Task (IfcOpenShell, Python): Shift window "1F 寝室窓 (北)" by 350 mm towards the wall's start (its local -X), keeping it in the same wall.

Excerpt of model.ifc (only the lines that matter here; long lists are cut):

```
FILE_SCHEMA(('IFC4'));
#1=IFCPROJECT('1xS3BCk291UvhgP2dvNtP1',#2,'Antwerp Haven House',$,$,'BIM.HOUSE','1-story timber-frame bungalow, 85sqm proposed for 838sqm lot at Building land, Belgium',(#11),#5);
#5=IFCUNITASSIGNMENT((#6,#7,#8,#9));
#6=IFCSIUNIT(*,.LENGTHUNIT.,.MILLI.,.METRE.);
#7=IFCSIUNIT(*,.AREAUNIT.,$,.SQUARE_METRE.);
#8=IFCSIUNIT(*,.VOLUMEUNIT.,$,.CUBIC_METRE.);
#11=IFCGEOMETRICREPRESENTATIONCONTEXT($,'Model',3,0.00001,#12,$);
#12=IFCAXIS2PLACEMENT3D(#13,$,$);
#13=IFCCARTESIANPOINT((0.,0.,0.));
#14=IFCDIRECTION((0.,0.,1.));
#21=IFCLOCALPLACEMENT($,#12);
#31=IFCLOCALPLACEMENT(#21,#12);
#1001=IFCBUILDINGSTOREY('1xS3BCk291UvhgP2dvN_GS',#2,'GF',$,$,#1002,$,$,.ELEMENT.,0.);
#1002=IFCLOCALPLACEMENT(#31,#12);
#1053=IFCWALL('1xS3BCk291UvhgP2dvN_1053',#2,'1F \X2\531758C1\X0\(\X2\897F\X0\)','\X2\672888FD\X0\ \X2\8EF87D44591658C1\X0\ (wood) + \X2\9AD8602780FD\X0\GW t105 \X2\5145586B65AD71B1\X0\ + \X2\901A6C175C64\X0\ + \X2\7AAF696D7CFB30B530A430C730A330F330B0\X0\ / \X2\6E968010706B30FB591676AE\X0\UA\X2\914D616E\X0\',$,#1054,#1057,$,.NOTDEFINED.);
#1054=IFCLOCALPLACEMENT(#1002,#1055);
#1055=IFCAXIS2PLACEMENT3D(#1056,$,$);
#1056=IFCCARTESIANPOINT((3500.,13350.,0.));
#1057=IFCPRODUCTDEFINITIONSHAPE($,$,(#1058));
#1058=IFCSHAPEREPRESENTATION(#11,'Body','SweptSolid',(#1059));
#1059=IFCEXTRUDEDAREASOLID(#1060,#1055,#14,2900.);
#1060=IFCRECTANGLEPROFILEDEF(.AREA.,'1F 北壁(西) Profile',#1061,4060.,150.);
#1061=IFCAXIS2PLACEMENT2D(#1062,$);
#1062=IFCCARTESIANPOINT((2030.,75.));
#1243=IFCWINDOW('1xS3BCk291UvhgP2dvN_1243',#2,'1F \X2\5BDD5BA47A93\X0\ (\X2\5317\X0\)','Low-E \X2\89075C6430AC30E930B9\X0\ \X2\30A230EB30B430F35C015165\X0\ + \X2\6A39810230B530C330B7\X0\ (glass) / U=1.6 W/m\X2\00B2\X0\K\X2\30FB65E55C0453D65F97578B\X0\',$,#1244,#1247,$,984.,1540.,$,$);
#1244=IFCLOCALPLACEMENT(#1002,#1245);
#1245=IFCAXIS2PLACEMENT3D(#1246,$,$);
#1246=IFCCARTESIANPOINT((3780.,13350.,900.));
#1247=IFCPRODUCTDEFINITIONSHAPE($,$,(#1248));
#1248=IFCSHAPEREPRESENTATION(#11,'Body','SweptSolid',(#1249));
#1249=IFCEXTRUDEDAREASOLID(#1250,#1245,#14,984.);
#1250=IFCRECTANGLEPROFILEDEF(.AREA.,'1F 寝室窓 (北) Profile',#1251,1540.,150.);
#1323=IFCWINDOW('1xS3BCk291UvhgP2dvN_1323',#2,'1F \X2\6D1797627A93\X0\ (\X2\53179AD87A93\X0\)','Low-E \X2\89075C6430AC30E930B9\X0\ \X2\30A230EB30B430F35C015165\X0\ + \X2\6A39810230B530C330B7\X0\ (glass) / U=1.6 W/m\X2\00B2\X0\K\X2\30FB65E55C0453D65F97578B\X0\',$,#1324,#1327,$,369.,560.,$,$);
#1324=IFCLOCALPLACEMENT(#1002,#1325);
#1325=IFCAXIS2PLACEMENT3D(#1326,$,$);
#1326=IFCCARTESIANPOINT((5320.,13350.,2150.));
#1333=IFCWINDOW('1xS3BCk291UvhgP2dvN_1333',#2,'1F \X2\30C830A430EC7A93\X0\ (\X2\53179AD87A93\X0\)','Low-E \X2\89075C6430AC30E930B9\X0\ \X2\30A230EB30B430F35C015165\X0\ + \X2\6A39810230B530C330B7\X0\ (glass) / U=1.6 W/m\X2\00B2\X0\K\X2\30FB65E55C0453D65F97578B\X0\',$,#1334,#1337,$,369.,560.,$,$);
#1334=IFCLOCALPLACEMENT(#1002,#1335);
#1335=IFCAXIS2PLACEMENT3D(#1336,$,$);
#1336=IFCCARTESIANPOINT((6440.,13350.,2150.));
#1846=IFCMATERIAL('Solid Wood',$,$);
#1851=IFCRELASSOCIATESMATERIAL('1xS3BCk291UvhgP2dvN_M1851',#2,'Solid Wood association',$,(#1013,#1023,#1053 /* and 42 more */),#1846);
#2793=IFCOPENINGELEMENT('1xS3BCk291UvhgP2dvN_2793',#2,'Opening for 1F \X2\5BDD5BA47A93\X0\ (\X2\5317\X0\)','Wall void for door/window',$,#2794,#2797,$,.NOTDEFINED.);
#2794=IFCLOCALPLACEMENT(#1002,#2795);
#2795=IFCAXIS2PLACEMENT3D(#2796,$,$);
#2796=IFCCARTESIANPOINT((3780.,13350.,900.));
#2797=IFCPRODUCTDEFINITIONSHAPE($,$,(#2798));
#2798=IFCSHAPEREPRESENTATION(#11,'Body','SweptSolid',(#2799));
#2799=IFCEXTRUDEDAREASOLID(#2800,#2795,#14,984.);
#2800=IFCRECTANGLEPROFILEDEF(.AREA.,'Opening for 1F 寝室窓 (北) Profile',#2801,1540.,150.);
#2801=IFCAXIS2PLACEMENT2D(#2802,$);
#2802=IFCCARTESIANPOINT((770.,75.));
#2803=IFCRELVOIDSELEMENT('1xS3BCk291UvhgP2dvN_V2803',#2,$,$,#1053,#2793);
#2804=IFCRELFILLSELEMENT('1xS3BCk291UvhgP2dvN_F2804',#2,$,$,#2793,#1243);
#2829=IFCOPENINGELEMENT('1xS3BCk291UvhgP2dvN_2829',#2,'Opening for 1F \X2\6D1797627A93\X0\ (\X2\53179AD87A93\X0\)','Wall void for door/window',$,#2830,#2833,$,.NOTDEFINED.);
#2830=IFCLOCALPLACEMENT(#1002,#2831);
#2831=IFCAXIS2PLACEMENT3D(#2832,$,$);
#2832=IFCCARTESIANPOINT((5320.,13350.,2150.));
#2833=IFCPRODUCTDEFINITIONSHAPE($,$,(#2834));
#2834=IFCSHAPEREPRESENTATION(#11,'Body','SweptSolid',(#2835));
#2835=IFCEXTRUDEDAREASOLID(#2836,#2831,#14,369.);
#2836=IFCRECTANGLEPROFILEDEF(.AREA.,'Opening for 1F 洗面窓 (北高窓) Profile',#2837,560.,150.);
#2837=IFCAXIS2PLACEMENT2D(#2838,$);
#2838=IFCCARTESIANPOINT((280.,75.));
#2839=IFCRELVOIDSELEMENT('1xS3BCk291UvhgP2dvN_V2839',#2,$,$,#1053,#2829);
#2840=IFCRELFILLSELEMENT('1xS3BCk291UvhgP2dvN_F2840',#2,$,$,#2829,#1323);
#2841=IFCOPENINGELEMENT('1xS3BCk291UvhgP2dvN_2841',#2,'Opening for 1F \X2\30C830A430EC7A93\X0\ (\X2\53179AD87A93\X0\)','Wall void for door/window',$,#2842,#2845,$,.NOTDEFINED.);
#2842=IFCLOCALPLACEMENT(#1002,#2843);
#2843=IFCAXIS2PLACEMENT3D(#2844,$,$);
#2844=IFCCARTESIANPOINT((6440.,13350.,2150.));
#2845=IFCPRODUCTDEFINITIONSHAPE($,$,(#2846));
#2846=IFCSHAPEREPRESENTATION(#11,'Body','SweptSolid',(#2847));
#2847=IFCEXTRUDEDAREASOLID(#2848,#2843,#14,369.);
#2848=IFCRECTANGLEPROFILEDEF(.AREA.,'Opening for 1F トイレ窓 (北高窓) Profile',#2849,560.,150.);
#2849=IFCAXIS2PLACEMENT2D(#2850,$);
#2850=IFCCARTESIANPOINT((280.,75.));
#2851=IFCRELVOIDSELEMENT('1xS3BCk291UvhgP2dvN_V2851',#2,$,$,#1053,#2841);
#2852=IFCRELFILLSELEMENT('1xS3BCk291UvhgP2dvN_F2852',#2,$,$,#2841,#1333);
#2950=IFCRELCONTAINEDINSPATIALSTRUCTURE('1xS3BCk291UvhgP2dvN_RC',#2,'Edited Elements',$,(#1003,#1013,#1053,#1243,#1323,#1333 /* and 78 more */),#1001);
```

```python
import ifcopenshell
import ifcopenshell.api.geometry
import ifcopenshell.util.placement
import ifcopenshell.util.unit

model = ifcopenshell.open("model.ifc")
unit_scale = ifcopenshell.util.unit.calculate_unit_scale(model)

window = model.by_guid("1xS3BCk291UvhgP2dvN_1243")
opening = window.FillsVoids[0].RelatingOpeningElement
wall = opening.VoidsElements[0].RelatingBuildingElement

wall_matrix = ifcopenshell.util.placement.get_local_placement(wall.ObjectPlacement)
shift = wall_matrix[:3, 0] * -0.35 / unit_scale
before = ifcopenshell.util.placement.get_local_placement(window.ObjectPlacement)[:3, 3].copy()

# The window is not placed relative to its opening, so move both.
for product in (opening, window):
    matrix = ifcopenshell.util.placement.get_local_placement(product.ObjectPlacement)
    matrix[:3, 3] += shift
    ifcopenshell.api.geometry.edit_object_placement(model, product=product, matrix=matrix, is_si=False)

after = ifcopenshell.util.placement.get_local_placement(window.ObjectPlacement)[:3, 3]
print("window moved by", (after - before).round(3) + 0.0)

model.write("model_v2.ifc")
```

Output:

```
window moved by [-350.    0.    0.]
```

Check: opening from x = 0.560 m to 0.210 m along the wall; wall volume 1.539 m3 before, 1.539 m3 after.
